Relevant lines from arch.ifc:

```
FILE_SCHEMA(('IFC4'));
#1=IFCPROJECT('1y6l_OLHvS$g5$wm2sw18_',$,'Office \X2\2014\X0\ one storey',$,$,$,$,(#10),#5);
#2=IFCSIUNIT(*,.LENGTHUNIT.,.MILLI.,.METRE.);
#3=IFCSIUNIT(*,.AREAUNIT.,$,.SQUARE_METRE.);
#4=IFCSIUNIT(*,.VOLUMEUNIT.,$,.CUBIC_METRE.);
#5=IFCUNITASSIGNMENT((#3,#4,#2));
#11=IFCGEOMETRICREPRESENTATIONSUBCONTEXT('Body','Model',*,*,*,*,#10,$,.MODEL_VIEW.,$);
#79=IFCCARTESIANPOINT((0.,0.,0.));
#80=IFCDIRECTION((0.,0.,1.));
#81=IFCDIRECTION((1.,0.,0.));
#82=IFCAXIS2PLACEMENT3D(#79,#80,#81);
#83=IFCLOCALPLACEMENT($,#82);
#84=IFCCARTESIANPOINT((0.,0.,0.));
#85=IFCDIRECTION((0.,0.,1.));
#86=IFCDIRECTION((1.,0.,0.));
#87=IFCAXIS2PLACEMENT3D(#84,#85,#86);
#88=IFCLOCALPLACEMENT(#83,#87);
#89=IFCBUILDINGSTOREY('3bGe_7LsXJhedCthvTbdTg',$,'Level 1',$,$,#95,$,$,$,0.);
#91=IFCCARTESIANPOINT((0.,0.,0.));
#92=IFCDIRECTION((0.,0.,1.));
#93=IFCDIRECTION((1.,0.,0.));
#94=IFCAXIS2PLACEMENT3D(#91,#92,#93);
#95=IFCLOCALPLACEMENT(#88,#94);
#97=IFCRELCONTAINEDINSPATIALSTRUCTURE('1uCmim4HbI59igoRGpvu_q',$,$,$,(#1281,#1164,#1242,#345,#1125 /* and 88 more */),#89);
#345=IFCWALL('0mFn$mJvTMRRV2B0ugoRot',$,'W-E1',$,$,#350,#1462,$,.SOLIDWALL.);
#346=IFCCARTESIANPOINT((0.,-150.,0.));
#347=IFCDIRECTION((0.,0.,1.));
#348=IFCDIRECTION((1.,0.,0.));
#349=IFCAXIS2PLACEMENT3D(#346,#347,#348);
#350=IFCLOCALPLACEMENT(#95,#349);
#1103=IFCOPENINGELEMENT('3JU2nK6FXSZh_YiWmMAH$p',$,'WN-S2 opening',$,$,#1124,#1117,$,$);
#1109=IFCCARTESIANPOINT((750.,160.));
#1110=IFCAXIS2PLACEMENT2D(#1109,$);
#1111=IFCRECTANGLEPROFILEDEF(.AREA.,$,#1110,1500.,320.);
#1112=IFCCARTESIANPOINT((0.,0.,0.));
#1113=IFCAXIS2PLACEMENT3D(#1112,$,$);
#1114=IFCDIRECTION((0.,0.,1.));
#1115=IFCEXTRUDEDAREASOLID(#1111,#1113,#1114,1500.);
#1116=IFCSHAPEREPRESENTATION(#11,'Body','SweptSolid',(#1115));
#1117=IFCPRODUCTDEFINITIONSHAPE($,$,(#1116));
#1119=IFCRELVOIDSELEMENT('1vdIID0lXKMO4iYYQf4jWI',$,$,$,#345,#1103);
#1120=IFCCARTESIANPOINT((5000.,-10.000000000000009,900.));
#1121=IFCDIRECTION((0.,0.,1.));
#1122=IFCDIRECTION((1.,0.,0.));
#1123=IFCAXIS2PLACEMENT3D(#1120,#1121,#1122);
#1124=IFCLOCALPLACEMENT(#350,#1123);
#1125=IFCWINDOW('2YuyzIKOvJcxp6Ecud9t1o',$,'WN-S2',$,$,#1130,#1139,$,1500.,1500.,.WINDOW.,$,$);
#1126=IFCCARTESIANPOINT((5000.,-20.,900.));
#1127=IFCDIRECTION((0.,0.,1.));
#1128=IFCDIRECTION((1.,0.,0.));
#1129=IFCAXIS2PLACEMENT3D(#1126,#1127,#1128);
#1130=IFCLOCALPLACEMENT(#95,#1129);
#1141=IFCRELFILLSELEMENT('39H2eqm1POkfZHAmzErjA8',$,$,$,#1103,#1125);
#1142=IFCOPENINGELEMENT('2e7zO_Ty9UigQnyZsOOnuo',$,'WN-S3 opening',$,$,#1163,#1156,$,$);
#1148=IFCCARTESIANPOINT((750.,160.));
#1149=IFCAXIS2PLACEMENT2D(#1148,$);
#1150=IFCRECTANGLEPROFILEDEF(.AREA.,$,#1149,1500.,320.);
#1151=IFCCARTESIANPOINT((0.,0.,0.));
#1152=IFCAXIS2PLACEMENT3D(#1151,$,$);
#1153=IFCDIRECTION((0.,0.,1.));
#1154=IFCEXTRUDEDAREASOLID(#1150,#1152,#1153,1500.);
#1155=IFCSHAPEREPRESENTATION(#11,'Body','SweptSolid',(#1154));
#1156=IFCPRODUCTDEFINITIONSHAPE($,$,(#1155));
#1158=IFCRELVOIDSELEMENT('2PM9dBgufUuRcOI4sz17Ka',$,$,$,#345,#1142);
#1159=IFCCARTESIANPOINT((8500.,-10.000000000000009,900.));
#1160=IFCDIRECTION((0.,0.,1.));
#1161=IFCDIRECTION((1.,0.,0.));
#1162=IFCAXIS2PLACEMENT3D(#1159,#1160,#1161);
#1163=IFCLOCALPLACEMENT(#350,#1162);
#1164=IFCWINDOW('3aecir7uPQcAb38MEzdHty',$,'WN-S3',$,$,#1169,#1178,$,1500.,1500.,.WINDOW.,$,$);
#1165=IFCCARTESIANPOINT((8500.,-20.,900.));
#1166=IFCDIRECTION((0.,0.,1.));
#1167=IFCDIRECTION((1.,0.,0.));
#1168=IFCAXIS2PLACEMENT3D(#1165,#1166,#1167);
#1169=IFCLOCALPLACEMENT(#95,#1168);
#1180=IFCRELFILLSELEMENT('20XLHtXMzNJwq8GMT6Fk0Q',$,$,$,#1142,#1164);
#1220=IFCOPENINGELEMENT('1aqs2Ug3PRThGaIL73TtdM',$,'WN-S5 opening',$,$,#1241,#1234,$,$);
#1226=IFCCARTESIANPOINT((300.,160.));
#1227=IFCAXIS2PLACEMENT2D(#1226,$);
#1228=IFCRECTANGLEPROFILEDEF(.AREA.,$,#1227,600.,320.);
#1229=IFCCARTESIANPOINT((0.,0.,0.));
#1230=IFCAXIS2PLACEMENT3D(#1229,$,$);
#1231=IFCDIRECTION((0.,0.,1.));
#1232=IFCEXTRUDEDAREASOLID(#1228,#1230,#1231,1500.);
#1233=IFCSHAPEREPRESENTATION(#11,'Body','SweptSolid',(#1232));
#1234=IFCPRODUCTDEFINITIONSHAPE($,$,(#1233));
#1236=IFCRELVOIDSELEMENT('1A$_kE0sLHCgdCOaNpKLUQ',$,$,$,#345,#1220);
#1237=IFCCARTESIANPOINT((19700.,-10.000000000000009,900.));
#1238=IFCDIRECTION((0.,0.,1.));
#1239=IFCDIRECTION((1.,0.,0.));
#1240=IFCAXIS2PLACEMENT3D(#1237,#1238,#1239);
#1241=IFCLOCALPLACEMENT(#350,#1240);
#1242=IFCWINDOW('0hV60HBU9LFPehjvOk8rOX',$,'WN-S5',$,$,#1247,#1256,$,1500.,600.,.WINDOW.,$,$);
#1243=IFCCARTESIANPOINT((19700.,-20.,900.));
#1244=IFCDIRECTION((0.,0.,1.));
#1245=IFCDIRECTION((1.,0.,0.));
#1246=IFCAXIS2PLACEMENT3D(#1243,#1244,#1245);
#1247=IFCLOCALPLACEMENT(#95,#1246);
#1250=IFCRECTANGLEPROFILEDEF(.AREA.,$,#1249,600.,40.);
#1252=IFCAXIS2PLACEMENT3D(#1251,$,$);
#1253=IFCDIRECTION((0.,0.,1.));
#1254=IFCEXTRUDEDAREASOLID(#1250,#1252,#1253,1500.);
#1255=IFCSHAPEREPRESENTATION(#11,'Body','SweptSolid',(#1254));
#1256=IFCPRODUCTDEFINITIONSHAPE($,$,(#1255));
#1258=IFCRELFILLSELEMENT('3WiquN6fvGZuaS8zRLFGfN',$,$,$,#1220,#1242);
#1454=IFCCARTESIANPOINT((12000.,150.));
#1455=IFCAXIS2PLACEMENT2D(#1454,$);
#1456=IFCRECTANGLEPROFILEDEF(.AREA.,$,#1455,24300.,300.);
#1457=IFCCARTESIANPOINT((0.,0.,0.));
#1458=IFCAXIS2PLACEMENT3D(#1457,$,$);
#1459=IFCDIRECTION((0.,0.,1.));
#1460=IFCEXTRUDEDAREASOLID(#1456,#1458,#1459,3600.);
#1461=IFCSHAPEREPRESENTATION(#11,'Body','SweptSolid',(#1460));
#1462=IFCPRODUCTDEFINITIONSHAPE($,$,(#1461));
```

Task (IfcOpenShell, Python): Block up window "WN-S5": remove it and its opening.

```python
import ifcopenshell
import ifcopenshell.api.feature
import ifcopenshell.api.root
import ifcopenshell.geom
import ifcopenshell.util.shape

model = ifcopenshell.open("arch.ifc")
settings = ifcopenshell.geom.settings()


def volume(element):
    """Net volume in cubic metres, openings subtracted."""
    shape = ifcopenshell.geom.create_shape(settings, element)
    return ifcopenshell.util.shape.get_volume(shape.geometry)


window = model.by_guid("0hV60HBU9LFPehjvOk8rOX")
opening = window.FillsVoids[0].RelatingOpeningElement
wall = opening.VoidsElements[0].RelatingBuildingElement
before = volume(wall)

ifcopenshell.api.root.remove_product(model, product=window)
ifcopenshell.api.feature.remove_feature(model, feature=opening)

after = volume(wall)

print(f"wall volume {before:.3f} -> {after:.3f} m3")

model.write("arch_v2.ifc")
```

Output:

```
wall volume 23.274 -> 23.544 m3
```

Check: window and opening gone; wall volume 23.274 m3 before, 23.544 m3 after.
